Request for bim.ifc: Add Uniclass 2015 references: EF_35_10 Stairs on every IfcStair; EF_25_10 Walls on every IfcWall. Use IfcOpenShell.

First a look at what the model holds.

```python
import ifcopenshell

model = ifcopenshell.open("bim.ifc")
print(model.schema)
print("classifications:", [c.Name for c in model.by_type("IfcClassification")])
for ifc_class in ("IfcDoor", "IfcRoof", "IfcStair", "IfcWall", "IfcWindow"):
    print(ifc_class, len(model.by_type(ifc_class)))
```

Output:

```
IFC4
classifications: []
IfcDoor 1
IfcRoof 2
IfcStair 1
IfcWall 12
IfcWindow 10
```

```python
import ifcopenshell
import ifcopenshell.api.classification

model = ifcopenshell.open("bim.ifc")

system = ifcopenshell.api.classification.add_classification(model, classification="Uniclass 2015")

codes = {
    "IfcStair": ("EF_35_10", "Stairs"),
    "IfcWall": ("EF_25_10", "Walls"),
}
for ifc_class, (code, name) in codes.items():
    products = model.by_type(ifc_class)
    ifcopenshell.api.classification.add_reference(
        model, products=products, classification=system, identification=code, name=name
    )
    print(code, len(products))

model.write("bim_edited.ifc")
```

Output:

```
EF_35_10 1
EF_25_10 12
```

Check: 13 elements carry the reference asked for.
